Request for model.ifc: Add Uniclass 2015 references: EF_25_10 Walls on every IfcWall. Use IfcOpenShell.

First a look at what the model holds.

```python
import ifcopenshell

model = ifcopenshell.open("model.ifc")
print(model.schema)
print("classifications:", [c.Name for c in model.by_type("IfcClassification")])
for ifc_class in ("IfcDoor", "IfcRoof", "IfcStair", "IfcWall", "IfcWindow"):
    print(ifc_class, len(model.by_type(ifc_class)))
```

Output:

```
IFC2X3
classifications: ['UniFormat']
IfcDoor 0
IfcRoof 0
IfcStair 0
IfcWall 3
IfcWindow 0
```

```python
import ifcopenshell
import ifcopenshell.api.classification

model = ifcopenshell.open("model.ifc")

# IFC2X3 requires Source and Edition and has no link from the project to the system.
system = model.create_entity("IfcClassification", Source="NBS", Edition="2015", Name="Uniclass 2015")

codes = {
    "IfcWall": ("EF_25_10", "Walls"),
}
for ifc_class, (code, name) in codes.items():
    products = model.by_type(ifc_class)
    ifcopenshell.api.classification.add_reference(
        model, products=products, classification=system, identification=code, name=name
    )
    print(code, len(products))

model.write("model_updated.ifc")
```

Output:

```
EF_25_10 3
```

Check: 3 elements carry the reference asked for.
